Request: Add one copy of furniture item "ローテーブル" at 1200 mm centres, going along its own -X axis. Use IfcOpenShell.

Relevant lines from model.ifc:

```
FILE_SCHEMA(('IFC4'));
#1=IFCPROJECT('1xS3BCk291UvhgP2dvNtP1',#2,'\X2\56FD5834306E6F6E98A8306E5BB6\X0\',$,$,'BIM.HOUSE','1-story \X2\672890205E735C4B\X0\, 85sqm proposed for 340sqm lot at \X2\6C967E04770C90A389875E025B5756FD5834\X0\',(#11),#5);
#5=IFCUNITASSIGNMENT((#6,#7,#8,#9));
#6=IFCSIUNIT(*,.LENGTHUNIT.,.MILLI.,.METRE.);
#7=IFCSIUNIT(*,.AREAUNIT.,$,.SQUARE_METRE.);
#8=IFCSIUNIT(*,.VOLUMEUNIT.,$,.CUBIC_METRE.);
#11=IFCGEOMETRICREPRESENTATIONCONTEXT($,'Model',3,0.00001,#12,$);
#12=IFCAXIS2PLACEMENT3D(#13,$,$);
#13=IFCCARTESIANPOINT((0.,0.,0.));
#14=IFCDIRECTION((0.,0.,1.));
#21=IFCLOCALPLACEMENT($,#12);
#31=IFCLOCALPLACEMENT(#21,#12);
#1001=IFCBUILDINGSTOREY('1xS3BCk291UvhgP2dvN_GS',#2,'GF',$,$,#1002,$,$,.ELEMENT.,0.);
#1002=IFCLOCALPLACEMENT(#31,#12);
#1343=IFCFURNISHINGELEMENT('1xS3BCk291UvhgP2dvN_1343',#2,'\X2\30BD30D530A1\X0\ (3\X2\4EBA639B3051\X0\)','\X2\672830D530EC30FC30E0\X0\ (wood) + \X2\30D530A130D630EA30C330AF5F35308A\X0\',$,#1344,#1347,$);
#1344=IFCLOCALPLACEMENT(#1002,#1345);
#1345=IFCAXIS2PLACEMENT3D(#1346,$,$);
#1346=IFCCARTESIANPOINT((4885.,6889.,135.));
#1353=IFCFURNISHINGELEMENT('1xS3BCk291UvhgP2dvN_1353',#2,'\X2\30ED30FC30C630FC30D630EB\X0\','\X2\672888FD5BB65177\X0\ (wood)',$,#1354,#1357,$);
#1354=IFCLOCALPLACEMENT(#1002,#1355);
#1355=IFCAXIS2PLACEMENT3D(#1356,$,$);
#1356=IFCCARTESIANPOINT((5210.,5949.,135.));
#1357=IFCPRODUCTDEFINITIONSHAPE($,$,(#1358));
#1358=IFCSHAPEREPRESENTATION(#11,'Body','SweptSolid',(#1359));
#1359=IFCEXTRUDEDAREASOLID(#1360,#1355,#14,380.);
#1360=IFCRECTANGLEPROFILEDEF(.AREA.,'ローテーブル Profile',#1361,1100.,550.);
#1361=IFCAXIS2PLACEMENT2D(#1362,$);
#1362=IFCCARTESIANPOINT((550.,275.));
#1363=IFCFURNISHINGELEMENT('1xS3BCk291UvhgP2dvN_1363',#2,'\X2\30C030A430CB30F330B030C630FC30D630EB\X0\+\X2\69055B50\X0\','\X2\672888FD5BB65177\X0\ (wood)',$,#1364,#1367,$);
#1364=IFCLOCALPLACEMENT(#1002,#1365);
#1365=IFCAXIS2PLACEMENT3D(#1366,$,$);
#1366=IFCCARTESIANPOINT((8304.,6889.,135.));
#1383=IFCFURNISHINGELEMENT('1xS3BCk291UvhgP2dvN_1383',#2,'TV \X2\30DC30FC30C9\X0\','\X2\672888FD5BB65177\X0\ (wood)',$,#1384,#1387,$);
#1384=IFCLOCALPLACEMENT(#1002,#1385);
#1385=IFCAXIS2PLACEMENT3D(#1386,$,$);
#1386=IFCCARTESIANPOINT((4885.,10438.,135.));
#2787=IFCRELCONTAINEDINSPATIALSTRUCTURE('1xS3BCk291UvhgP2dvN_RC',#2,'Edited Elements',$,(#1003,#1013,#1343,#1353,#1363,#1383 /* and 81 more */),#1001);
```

```python
import ifcopenshell
import ifcopenshell.api.geometry
import ifcopenshell.api.root
import ifcopenshell.util.element
import ifcopenshell.util.placement

model = ifcopenshell.open("model.ifc")


def reuse_history(source, copy):
    """copy_class also copies each property set's owner history, people and application; keep the originals."""
    for rel in copy.IsDefinedBy:
        if rel.is_a("IfcRelDefinesByProperties") and (history := rel.RelatingPropertyDefinition.OwnerHistory):
            rel.RelatingPropertyDefinition.OwnerHistory = source.OwnerHistory
            ifcopenshell.util.element.remove_deep2(model, history)


source = model.by_guid("1xS3BCk291UvhgP2dvN_1353")
base = ifcopenshell.util.placement.get_local_placement(source.ObjectPlacement)
step = -base[:3, 0] * 1200.0

for i in range(1, 2):
    copy = ifcopenshell.api.root.copy_class(model, product=source)
    copy.Representation = ifcopenshell.util.element.copy_deep(
        model, source.Representation, exclude=["IfcGeometricRepresentationContext", "IfcRepresentationMap"]
    )
    reuse_history(source, copy)
    matrix = base.copy()
    matrix[:3, 3] += i * step
    print("added at", matrix[:3, 3].round(3) + 0.0)
    ifcopenshell.api.geometry.edit_object_placement(model, product=copy, matrix=matrix, is_si=False)

model.write("model_v2.ifc")
```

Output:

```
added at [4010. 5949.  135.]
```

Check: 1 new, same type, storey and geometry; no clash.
